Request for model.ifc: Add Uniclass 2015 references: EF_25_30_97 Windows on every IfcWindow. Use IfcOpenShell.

First a look at what the model holds.

```python
import ifcopenshell

model = ifcopenshell.open("model.ifc")
print(model.schema)
print("classifications:", [c.Name for c in model.by_type("IfcClassification")])
for ifc_class in ("IfcDoor", "IfcRoof", "IfcStair", "IfcWall", "IfcWindow"):
    print(ifc_class, len(model.by_type(ifc_class)))
```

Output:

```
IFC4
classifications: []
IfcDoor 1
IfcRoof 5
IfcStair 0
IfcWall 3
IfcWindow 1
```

```python
import ifcopenshell
import ifcopenshell.api.classification

model = ifcopenshell.open("model.ifc")

system = ifcopenshell.api.classification.add_classification(model, classification="Uniclass 2015")

codes = {
    "IfcWindow": ("EF_25_30_97", "Windows"),
}
for ifc_class, (code, name) in codes.items():
    products = model.by_type(ifc_class)
    ifcopenshell.api.classification.add_reference(
        model, products=products, classification=system, identification=code, name=name
    )
    print(code, len(products))

model.write("model_edited.ifc")
```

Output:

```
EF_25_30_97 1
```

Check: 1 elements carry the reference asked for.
